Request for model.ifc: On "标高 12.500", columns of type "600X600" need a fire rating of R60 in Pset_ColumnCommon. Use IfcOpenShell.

First a look at what the model holds.

```python
import ifcopenshell
import ifcopenshell.util.element

model = ifcopenshell.open("model.ifc")
print(model.schema)
storey = next(s for s in model.by_type("IfcBuildingStorey") if s.Name == "标高 12.500")
columns = [e for e in ifcopenshell.util.element.get_decomposition(storey) if e.is_a("IfcColumn")]
seen = {}
for e in columns:
    element_type = ifcopenshell.util.element.get_type(e)
    key = (element_type.Name if element_type != e and element_type else None, ifcopenshell.util.element.get_pset(e, "Pset_ColumnCommon", "FireRating"))
    seen[key] = seen.get(key, 0) + 1
for (name, value), count in sorted(seen.items(), key=str):
    print(count, "x", name, "|", value)
```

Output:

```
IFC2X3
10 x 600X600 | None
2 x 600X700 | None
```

```python
import ifcopenshell
import ifcopenshell.api.pset
import ifcopenshell.util.element

model = ifcopenshell.open("model.ifc")

storey = next(s for s in model.by_type("IfcBuildingStorey") if s.Name == "标高 12.500")
columns = [e for e in ifcopenshell.util.element.get_decomposition(storey) if e.is_a("IfcColumn")]

count = 0
for e in columns:
    element_type = ifcopenshell.util.element.get_type(e)
    if element_type in (None, e) or element_type.Name != "600X600":
        continue
    # add_pset returns the element's existing set when there is one.
    pset = ifcopenshell.api.pset.add_pset(model, product=e, name="Pset_ColumnCommon")
    ifcopenshell.api.pset.edit_pset(model, pset=pset, properties={"FireRating": "R60"})
    count += 1

print(count, "columns updated")

model.write("model_edited.ifc")
```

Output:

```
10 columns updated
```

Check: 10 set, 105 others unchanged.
